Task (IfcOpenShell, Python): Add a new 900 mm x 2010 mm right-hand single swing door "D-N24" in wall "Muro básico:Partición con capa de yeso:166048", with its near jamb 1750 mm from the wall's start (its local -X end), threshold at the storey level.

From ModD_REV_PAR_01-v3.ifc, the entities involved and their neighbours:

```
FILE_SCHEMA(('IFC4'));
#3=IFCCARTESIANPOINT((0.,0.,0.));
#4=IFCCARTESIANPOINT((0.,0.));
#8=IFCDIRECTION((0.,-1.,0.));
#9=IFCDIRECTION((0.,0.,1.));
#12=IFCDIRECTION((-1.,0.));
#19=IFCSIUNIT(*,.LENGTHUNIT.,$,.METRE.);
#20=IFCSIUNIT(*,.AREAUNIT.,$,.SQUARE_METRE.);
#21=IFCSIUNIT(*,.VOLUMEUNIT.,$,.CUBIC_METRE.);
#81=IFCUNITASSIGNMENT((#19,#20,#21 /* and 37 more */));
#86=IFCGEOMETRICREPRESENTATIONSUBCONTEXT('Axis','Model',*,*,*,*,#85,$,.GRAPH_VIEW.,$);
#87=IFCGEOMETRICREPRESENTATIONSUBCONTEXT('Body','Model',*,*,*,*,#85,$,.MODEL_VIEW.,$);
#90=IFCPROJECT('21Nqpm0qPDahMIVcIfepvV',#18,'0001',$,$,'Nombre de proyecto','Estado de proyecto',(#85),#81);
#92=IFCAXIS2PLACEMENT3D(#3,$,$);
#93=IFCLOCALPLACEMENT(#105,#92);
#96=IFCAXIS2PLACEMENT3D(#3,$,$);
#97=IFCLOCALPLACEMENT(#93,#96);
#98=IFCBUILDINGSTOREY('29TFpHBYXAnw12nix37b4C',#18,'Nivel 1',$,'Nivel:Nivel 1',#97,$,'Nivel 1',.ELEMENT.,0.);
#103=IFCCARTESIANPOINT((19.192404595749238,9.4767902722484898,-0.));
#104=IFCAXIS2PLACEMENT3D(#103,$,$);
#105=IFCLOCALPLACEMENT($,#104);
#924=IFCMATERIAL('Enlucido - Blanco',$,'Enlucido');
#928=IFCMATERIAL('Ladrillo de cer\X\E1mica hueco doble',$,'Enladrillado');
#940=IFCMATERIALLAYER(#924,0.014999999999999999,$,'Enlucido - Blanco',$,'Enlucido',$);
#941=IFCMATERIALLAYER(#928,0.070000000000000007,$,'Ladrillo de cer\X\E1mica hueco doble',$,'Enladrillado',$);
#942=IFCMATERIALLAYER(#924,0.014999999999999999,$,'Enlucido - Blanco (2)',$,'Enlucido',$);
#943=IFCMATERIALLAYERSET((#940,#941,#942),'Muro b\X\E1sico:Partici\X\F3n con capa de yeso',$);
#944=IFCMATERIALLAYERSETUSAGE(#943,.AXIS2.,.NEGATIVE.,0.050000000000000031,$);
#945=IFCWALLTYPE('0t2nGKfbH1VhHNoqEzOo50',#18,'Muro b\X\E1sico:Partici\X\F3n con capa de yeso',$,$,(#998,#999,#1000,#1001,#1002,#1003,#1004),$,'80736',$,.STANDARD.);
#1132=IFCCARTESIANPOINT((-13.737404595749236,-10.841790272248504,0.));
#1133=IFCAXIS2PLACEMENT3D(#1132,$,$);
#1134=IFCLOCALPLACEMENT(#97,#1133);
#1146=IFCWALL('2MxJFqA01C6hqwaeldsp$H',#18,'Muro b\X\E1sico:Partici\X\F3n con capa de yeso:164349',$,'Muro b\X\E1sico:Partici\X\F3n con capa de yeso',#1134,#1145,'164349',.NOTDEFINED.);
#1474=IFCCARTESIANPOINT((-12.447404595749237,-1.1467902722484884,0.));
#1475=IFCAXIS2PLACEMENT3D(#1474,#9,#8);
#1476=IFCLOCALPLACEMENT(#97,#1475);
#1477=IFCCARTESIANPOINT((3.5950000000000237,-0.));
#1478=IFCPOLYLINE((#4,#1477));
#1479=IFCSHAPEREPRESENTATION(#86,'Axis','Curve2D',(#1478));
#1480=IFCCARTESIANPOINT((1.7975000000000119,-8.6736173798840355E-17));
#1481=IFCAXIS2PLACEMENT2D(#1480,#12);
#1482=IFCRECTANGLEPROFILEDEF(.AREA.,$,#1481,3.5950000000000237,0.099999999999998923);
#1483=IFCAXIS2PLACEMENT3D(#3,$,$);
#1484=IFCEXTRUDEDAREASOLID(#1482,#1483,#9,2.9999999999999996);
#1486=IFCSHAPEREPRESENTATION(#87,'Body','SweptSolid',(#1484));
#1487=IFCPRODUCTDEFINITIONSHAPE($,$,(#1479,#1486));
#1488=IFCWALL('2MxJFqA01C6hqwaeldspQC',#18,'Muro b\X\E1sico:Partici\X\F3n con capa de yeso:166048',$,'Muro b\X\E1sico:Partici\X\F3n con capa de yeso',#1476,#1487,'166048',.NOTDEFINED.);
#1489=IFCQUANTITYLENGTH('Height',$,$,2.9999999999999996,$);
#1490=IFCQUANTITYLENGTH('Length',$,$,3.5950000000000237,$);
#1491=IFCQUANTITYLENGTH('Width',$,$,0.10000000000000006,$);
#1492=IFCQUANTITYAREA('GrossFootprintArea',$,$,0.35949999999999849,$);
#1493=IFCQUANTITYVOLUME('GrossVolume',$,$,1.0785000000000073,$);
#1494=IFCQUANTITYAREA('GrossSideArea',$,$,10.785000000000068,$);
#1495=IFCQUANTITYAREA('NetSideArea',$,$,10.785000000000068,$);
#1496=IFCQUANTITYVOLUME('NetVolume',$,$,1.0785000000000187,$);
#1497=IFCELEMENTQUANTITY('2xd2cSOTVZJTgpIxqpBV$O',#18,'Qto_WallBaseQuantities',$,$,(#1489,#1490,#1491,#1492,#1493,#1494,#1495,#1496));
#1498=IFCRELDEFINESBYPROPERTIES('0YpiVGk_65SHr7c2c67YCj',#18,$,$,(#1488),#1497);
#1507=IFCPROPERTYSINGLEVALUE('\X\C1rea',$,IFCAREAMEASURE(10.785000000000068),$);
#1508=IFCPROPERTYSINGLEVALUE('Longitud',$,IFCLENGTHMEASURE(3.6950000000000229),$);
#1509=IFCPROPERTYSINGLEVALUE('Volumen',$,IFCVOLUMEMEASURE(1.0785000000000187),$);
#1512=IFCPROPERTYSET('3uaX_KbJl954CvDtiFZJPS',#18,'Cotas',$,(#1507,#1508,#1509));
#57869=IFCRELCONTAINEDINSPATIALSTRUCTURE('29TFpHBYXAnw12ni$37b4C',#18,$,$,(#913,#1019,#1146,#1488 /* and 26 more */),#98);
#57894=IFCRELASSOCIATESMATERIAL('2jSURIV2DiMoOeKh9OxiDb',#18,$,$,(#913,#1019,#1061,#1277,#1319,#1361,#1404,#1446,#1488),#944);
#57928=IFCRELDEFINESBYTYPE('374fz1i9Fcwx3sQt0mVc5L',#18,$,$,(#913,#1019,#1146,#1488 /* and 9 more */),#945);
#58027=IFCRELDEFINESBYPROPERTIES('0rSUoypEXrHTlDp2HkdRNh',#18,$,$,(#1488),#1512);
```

```python
import numpy as np
import ifcopenshell
import ifcopenshell.api.feature
import ifcopenshell.api.geometry
import ifcopenshell.api.pset
import ifcopenshell.api.root
import ifcopenshell.api.spatial
import ifcopenshell.geom
import ifcopenshell.util.element
import ifcopenshell.util.placement
import ifcopenshell.util.representation
import ifcopenshell.util.shape
import ifcopenshell.util.unit

model = ifcopenshell.open("ModD_REV_PAR_01-v3.ifc")
unit_scale = ifcopenshell.util.unit.calculate_unit_scale(model)
area_scale = ifcopenshell.util.unit.calculate_unit_scale(model, "AREAUNIT")
volume_scale = ifcopenshell.util.unit.calculate_unit_scale(model, "VOLUMEUNIT")
settings = ifcopenshell.geom.settings()


def volume(element):
    """Net volume in cubic metres, openings subtracted."""
    shape = ifcopenshell.geom.create_shape(settings, element)
    return ifcopenshell.util.shape.get_volume(shape.geometry)


wall = model.by_guid("2MxJFqA01C6hqwaeldspQC")
storey = ifcopenshell.util.element.get_container(wall, ifc_class="IfcBuildingStorey")
context = ifcopenshell.util.representation.get_context(model, "Model", "Body", "MODEL_VIEW")
before = volume(wall)

width, height, from_end, sill = 0.9, 2.01, 1.75, 0.0  # metres

# The wall runs along its own X axis, and the end named is its -X end.
wall_shape = ifcopenshell.geom.create_shape(settings, wall)
x, y, z = ifcopenshell.util.shape.get_vertices(wall_shape.geometry).T
start = x.min() + from_end
face, thickness = float(y.min()), float(y.max() - y.min())
wall_matrix = ifcopenshell.util.placement.get_local_placement(wall.ObjectPlacement)
level = ifcopenshell.util.placement.get_local_placement(storey.ObjectPlacement)[2, 3]


def in_wall(x, y):
    """Placement at x, y metres in the wall's axes, at sill height."""
    matrix = wall_matrix.copy()
    matrix[:, 3] = wall_matrix @ np.array([x / unit_scale, y / unit_scale, 0.0, 1.0])
    matrix[2, 3] = level + sill / unit_scale
    return matrix


# Opening: a box that overshoots both wall faces by 50 mm.
opening = ifcopenshell.api.root.create_entity(model, ifc_class="IfcOpeningElement", predefined_type="OPENING")
box = ifcopenshell.api.geometry.add_wall_representation(
    model, context=context, length=width, height=height, thickness=thickness + 0.1
)
ifcopenshell.api.geometry.assign_representation(model, product=opening, representation=box)
ifcopenshell.api.geometry.edit_object_placement(model, product=opening, matrix=in_wall(start, face - 0.05), is_si=False)
ifcopenshell.api.feature.add_feature(model, feature=opening, element=wall)

door = ifcopenshell.api.root.create_entity(model, ifc_class="IfcDoor", name="D-N24", predefined_type="DOOR")
door.OverallWidth, door.OverallHeight = width / unit_scale, height / unit_scale
door.OperationType = "SINGLE_SWING_RIGHT"
body = ifcopenshell.api.geometry.add_door_representation(
    model,
    context=context,
    overall_width=door.OverallWidth,
    overall_height=door.OverallHeight,
    operation_type="SINGLE_SWING_RIGHT",
    lining_properties={"LiningDepth": thickness / unit_scale, "ThresholdDepth": thickness / unit_scale},
)
ifcopenshell.api.geometry.assign_representation(model, product=door, representation=body)
ifcopenshell.api.spatial.assign_container(model, products=[door], relating_structure=storey)
ifcopenshell.api.feature.add_filling(model, opening=opening, element=door)

# The lining spans the wall, so the door starts at the wall face.
ifcopenshell.api.geometry.edit_object_placement(model, product=door, matrix=in_wall(start, face), is_si=False)

after = volume(wall)

# Update the wall's stored quantities.
qto = model.by_id(ifcopenshell.util.element.get_pset(wall, "Qto_WallBaseQuantities", should_inherit=False)["id"])
ifcopenshell.api.pset.edit_qto(model, qto=qto, properties={
    "NetSideArea": after / thickness / area_scale,
    "NetVolume": after / volume_scale,
})
pset = model.by_id(ifcopenshell.util.element.get_pset(wall, "Cotas", should_inherit=False)["id"])
ifcopenshell.api.pset.edit_pset(model, pset=pset, properties={
    "Área": model.create_entity("IfcAreaMeasure", after / thickness / area_scale),
    "Volumen": model.create_entity("IfcVolumeMeasure", after / volume_scale),
})

print(f"wall volume {before:.3f} -> {after:.3f} m3")

model.write("ModD_REV_PAR_01-v3_rev.ifc")
```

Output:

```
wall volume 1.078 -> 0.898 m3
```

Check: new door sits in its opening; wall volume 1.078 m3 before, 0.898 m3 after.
